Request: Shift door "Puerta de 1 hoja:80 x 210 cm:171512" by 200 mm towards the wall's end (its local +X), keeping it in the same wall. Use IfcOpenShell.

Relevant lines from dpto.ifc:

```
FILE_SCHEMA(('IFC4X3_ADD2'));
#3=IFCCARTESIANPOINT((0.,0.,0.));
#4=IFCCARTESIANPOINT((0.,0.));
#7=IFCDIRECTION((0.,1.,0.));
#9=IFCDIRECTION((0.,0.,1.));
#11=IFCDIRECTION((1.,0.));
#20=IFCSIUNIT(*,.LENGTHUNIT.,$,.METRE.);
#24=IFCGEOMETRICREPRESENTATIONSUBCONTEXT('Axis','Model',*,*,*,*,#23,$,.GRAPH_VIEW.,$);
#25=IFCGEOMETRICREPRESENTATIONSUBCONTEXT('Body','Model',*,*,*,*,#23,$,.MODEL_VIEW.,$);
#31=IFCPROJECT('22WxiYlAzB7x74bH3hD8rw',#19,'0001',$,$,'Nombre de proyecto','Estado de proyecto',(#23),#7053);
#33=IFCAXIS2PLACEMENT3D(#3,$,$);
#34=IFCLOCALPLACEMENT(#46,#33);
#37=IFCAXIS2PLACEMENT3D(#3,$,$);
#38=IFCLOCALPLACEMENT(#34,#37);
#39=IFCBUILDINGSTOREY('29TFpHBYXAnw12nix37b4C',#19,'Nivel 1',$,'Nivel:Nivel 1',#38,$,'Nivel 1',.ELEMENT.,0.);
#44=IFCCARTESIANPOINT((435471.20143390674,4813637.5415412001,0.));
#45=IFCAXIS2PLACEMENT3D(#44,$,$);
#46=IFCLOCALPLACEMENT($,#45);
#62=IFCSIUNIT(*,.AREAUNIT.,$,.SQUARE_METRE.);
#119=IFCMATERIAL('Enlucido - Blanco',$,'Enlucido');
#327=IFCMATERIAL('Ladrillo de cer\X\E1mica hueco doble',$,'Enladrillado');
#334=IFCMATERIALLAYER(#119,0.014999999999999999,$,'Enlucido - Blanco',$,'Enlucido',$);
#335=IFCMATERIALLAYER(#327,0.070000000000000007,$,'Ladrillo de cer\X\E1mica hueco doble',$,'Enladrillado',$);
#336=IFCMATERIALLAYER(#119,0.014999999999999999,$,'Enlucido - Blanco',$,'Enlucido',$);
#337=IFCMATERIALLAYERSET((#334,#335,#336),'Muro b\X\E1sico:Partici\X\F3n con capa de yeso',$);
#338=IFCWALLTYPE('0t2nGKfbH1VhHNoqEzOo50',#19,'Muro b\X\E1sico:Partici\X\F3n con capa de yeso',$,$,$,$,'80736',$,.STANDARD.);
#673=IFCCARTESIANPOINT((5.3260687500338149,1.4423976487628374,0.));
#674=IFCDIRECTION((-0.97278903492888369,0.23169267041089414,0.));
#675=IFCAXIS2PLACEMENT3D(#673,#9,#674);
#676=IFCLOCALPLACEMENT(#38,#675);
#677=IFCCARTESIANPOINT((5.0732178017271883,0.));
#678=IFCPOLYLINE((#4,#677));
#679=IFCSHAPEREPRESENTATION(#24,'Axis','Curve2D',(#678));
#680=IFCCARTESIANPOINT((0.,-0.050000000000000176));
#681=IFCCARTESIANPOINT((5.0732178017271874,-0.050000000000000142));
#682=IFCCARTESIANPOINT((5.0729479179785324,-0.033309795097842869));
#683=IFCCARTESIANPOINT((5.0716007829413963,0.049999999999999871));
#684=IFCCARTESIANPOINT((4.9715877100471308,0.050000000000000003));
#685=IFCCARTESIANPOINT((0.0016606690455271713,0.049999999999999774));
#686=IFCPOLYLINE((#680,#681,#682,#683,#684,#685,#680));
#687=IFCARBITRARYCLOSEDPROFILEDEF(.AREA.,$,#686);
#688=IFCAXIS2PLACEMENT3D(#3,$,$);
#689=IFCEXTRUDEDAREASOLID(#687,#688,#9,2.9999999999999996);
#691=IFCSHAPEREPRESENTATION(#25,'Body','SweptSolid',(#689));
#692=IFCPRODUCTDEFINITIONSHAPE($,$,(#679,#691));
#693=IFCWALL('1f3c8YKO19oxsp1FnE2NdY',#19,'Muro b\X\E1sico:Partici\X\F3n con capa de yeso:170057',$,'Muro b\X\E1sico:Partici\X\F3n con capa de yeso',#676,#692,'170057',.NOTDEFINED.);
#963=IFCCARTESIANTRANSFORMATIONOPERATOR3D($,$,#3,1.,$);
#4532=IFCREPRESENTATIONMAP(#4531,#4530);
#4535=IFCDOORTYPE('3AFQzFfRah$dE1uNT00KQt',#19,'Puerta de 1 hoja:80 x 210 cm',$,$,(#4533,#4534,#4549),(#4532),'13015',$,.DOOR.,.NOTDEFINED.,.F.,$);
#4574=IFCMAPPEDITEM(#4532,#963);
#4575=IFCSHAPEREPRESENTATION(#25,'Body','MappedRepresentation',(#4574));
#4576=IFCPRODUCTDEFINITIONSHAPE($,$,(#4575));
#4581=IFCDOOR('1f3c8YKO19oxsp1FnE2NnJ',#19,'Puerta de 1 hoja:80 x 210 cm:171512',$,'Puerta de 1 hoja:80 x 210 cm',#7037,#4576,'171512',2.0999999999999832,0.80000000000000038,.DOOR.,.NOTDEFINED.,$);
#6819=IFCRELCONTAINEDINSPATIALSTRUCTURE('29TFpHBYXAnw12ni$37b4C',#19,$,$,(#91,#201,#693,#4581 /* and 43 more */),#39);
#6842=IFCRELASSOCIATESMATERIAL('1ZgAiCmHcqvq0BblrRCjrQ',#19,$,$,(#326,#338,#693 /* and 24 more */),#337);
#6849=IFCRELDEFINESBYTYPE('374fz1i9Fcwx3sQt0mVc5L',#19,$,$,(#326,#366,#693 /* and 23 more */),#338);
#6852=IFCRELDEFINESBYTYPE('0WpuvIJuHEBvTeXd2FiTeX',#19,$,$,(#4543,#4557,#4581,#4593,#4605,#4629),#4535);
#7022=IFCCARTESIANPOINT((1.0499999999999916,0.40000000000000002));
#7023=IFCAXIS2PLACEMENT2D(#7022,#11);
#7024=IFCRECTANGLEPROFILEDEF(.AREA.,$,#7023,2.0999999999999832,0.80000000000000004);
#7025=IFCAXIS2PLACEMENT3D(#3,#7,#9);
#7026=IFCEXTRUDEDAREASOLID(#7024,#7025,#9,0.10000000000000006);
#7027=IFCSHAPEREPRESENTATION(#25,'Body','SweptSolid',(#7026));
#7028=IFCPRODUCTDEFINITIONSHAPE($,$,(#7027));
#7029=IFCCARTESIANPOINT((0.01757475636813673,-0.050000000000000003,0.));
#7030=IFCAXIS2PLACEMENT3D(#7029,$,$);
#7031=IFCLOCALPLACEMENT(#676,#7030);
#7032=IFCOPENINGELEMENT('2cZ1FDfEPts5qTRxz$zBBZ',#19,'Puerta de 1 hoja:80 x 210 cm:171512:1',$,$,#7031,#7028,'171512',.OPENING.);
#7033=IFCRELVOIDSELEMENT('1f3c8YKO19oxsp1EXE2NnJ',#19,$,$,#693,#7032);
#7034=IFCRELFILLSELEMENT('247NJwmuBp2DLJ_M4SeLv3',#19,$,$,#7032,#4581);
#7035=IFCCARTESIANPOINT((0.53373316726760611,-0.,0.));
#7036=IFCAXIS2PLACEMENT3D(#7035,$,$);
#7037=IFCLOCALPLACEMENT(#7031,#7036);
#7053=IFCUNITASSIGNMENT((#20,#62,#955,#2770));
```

```python
import ifcopenshell
import ifcopenshell.api.geometry
import ifcopenshell.util.placement
import ifcopenshell.util.unit

model = ifcopenshell.open("dpto.ifc")
unit_scale = ifcopenshell.util.unit.calculate_unit_scale(model)

door = model.by_id(4581)
opening = door.FillsVoids[0].RelatingOpeningElement
wall = opening.VoidsElements[0].RelatingBuildingElement

wall_matrix = ifcopenshell.util.placement.get_local_placement(wall.ObjectPlacement)
shift = wall_matrix[:3, 0] * 0.2 / unit_scale
before = ifcopenshell.util.placement.get_local_placement(door.ObjectPlacement)[:3, 3].copy()

# The door is placed relative to its opening, so it follows when the opening moves.
matrix = ifcopenshell.util.placement.get_local_placement(opening.ObjectPlacement)
matrix[:3, 3] += shift
ifcopenshell.api.geometry.edit_object_placement(
    model, product=opening, matrix=matrix, is_si=False, should_transform_children=True
)

after = ifcopenshell.util.placement.get_local_placement(door.ObjectPlacement)[:3, 3]
print("door moved by", (after - before).round(3) + 0.0)

model.write("dpto_v2.ifc")
```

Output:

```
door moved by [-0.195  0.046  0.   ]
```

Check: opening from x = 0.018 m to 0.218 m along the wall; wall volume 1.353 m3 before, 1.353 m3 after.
